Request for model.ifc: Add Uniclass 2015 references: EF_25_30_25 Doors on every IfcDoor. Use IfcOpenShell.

First a look at what the model holds.

```python
import ifcopenshell

model = ifcopenshell.open("model.ifc")
print(model.schema)
print("classifications:", [c.Name for c in model.by_type("IfcClassification")])
for ifc_class in ("IfcDoor", "IfcRoof", "IfcStair", "IfcWall", "IfcWindow"):
    print(ifc_class, len(model.by_type(ifc_class)))
```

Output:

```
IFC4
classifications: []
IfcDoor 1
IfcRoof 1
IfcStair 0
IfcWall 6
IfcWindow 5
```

```python
import ifcopenshell
import ifcopenshell.api.classification

model = ifcopenshell.open("model.ifc")

system = ifcopenshell.api.classification.add_classification(model, classification="Uniclass 2015")

codes = {
    "IfcDoor": ("EF_25_30_25", "Doors"),
}
for ifc_class, (code, name) in codes.items():
    products = model.by_type(ifc_class)
    ifcopenshell.api.classification.add_reference(
        model, products=products, classification=system, identification=code, name=name
    )
    print(code, len(products))

model.write("model_rev.ifc")
```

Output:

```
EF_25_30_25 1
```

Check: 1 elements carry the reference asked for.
